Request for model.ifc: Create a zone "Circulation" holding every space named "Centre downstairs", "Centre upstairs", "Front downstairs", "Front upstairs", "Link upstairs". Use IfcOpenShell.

First a look at what the model holds.

```python
import ifcopenshell

model = ifcopenshell.open("model.ifc")
print(model.schema)
seen = {}
for space in model.by_type("IfcSpace"):
    seen[space.Name] = seen.get(space.Name, 0) + 1
for name, count in sorted(seen.items(), key=str):
    print(count, "x", name)
print("zones:", [z.Name for z in model.by_type("IfcZone")][:20])
```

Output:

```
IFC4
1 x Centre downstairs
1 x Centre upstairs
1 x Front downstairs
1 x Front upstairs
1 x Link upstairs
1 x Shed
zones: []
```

```python
import ifcopenshell
import ifcopenshell.api.group
import ifcopenshell.api.root

model = ifcopenshell.open("model.ifc")

names = {"Centre downstairs", "Centre upstairs", "Front downstairs", "Front upstairs", "Link upstairs"}
spaces = [s for s in model.by_type("IfcSpace") if s.Name in names]

zone = ifcopenshell.api.root.create_entity(model, ifc_class="IfcZone", name="Circulation")
ifcopenshell.api.group.assign_group(model, products=spaces, group=zone)
print(len(spaces), "spaces in", zone.Name)

model.write("model_edited.ifc")
```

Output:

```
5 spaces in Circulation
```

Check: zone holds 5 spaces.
